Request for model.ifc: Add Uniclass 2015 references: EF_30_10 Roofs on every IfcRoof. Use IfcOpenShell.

First a look at what the model holds.

```python
import ifcopenshell

model = ifcopenshell.open("model.ifc")
print(model.schema)
print("classifications:", [c.Name for c in model.by_type("IfcClassification")])
for ifc_class in ("IfcDoor", "IfcRoof", "IfcStair", "IfcWall", "IfcWindow"):
    print(ifc_class, len(model.by_type(ifc_class)))
```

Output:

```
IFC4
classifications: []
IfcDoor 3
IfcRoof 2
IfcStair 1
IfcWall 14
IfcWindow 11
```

```python
import ifcopenshell
import ifcopenshell.api.classification

model = ifcopenshell.open("model.ifc")

system = ifcopenshell.api.classification.add_classification(model, classification="Uniclass 2015")

codes = {
    "IfcRoof": ("EF_30_10", "Roofs"),
}
for ifc_class, (code, name) in codes.items():
    products = model.by_type(ifc_class)
    ifcopenshell.api.classification.add_reference(
        model, products=products, classification=system, identification=code, name=name
    )
    print(code, len(products))

model.write("model_updated.ifc")
```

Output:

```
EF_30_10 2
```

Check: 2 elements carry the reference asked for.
